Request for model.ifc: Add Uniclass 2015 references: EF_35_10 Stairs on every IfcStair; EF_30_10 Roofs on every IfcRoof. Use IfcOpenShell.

First a look at what the model holds.

```python
import ifcopenshell

model = ifcopenshell.open("model.ifc")
print(model.schema)
print("classifications:", [c.Name for c in model.by_type("IfcClassification")])
for ifc_class in ("IfcDoor", "IfcRoof", "IfcStair", "IfcWall", "IfcWindow"):
    print(ifc_class, len(model.by_type(ifc_class)))
```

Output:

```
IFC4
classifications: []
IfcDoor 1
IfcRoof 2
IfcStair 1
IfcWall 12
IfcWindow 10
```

```python
import ifcopenshell
import ifcopenshell.api.classification

model = ifcopenshell.open("model.ifc")

system = ifcopenshell.api.classification.add_classification(model, classification="Uniclass 2015")

codes = {
    "IfcStair": ("EF_35_10", "Stairs"),
    "IfcRoof": ("EF_30_10", "Roofs"),
}
for ifc_class, (code, name) in codes.items():
    products = model.by_type(ifc_class)
    ifcopenshell.api.classification.add_reference(
        model, products=products, classification=system, identification=code, name=name
    )
    print(code, len(products))

model.write("model_edited.ifc")
```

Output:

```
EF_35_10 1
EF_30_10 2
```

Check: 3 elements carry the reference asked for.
